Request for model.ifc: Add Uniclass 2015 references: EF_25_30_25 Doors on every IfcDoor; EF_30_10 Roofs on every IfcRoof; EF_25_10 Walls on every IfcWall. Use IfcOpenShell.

First a look at what the model holds.

```python
import ifcopenshell

model = ifcopenshell.open("model.ifc")
print(model.schema)
print("classifications:", [c.Name for c in model.by_type("IfcClassification")])
for ifc_class in ("IfcDoor", "IfcRoof", "IfcStair", "IfcWall", "IfcWindow"):
    print(ifc_class, len(model.by_type(ifc_class)))
```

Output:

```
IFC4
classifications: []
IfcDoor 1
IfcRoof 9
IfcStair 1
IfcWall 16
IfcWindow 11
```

```python
import ifcopenshell
import ifcopenshell.api.classification

model = ifcopenshell.open("model.ifc")

system = ifcopenshell.api.classification.add_classification(model, classification="Uniclass 2015")

codes = {
    "IfcDoor": ("EF_25_30_25", "Doors"),
    "IfcRoof": ("EF_30_10", "Roofs"),
    "IfcWall": ("EF_25_10", "Walls"),
}
for ifc_class, (code, name) in codes.items():
    products = model.by_type(ifc_class)
    ifcopenshell.api.classification.add_reference(
        model, products=products, classification=system, identification=code, name=name
    )
    print(code, len(products))

model.write("model_v2.ifc")
```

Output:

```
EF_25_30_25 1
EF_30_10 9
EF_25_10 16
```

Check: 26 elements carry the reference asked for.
